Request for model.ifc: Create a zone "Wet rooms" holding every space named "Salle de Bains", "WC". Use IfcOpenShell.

First a look at what the model holds.

```python
import ifcopenshell

model = ifcopenshell.open("model.ifc")
print(model.schema)
seen = {}
for space in model.by_type("IfcSpace"):
    seen[space.LongName] = seen.get(space.LongName, 0) + 1
for name, count in sorted(seen.items(), key=str):
    print(count, "x", name)
print("zones:", [z.Name for z in model.by_type("IfcZone")][:20])
```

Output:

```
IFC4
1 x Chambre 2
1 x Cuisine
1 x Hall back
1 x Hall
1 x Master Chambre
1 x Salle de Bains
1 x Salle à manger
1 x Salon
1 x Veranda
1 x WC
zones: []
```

```python
import ifcopenshell
import ifcopenshell.api.group
import ifcopenshell.api.root

model = ifcopenshell.open("model.ifc")

names = {"Salle de Bains", "WC"}
spaces = [s for s in model.by_type("IfcSpace") if s.LongName in names]

zone = ifcopenshell.api.root.create_entity(model, ifc_class="IfcZone", name="Wet rooms")
ifcopenshell.api.group.assign_group(model, products=spaces, group=zone)
print(len(spaces), "spaces in", zone.Name)

model.write("model_updated.ifc")
```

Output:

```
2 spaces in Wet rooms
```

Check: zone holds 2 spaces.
